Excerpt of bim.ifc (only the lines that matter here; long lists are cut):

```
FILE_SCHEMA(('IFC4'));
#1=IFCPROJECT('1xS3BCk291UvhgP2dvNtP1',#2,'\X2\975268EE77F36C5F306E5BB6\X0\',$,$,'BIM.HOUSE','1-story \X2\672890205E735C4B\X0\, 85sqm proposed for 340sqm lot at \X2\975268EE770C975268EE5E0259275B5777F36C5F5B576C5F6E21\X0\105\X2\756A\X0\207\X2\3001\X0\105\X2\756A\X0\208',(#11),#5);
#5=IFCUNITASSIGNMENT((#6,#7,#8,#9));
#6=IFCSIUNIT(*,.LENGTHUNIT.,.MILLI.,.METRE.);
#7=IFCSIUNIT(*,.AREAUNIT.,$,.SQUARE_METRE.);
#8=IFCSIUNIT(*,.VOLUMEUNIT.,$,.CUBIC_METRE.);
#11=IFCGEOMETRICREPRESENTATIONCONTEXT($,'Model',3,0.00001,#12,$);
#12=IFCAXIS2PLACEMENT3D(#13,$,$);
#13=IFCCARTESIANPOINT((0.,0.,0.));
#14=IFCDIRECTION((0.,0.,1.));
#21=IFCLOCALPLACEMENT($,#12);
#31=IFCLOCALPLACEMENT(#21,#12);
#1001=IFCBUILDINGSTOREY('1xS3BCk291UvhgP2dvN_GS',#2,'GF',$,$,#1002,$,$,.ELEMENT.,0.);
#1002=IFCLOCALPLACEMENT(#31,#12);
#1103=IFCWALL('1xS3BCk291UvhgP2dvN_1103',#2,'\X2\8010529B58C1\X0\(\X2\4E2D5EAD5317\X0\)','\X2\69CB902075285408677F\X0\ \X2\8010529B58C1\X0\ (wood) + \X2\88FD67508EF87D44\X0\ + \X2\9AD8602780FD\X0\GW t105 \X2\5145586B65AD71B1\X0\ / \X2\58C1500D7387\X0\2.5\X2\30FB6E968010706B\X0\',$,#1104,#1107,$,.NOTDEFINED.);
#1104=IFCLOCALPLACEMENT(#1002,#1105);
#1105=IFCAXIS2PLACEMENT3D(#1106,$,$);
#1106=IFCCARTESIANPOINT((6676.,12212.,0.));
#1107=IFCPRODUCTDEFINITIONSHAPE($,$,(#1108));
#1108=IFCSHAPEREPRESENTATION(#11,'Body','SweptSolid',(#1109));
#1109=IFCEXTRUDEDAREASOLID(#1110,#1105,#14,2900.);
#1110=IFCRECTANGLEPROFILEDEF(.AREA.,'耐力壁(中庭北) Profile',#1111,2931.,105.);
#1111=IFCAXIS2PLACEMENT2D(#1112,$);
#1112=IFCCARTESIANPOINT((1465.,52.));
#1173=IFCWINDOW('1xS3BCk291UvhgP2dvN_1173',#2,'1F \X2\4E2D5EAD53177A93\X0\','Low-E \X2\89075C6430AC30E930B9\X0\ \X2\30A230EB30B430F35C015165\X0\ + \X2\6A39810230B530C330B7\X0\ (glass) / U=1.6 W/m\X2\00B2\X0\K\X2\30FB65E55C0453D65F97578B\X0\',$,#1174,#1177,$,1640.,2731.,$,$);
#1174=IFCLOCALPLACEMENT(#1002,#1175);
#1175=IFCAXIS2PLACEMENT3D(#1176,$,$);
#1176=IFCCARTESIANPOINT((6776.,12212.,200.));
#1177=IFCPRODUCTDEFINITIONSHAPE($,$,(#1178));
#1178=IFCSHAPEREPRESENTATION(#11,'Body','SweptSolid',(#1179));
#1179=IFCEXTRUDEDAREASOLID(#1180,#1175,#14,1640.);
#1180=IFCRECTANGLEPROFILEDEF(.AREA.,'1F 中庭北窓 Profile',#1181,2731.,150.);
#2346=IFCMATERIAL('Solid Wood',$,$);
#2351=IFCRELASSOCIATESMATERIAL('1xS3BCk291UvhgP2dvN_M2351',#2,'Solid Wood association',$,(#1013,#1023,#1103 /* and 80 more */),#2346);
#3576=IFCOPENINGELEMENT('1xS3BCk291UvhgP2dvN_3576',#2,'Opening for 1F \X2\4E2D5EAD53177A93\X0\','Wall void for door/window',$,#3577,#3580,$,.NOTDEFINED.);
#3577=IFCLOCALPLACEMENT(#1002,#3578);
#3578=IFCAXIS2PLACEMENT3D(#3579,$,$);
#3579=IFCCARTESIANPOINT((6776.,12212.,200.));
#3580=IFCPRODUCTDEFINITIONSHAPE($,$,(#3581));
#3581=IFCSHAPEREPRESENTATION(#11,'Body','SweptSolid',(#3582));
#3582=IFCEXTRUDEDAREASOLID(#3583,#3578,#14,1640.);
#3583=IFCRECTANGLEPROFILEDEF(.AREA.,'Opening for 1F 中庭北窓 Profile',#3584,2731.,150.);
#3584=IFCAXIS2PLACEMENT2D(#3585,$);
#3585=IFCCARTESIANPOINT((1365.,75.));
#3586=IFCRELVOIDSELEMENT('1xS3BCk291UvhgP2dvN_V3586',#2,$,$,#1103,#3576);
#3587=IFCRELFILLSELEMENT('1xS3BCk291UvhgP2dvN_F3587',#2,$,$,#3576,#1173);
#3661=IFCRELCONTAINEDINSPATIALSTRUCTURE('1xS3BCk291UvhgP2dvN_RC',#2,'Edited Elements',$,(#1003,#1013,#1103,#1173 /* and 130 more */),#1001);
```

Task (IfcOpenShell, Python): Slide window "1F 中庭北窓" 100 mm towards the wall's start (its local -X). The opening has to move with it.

```python
import ifcopenshell
import ifcopenshell.api.geometry
import ifcopenshell.util.placement
import ifcopenshell.util.unit

model = ifcopenshell.open("bim.ifc")
unit_scale = ifcopenshell.util.unit.calculate_unit_scale(model)

window = model.by_guid("1xS3BCk291UvhgP2dvN_1173")
opening = window.FillsVoids[0].RelatingOpeningElement
wall = opening.VoidsElements[0].RelatingBuildingElement

wall_matrix = ifcopenshell.util.placement.get_local_placement(wall.ObjectPlacement)
shift = wall_matrix[:3, 0] * -0.1 / unit_scale
before = ifcopenshell.util.placement.get_local_placement(window.ObjectPlacement)[:3, 3].copy()

# The window is not placed relative to its opening, so move both.
for product in (opening, window):
    matrix = ifcopenshell.util.placement.get_local_placement(product.ObjectPlacement)
    matrix[:3, 3] += shift
    ifcopenshell.api.geometry.edit_object_placement(model, product=product, matrix=matrix, is_si=False)

after = ifcopenshell.util.placement.get_local_placement(window.ObjectPlacement)[:3, 3]
print("window moved by", (after - before).round(3) + 0.0)

model.write("bim-out.ifc")
```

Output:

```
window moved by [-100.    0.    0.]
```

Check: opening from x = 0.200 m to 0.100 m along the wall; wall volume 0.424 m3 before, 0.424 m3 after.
